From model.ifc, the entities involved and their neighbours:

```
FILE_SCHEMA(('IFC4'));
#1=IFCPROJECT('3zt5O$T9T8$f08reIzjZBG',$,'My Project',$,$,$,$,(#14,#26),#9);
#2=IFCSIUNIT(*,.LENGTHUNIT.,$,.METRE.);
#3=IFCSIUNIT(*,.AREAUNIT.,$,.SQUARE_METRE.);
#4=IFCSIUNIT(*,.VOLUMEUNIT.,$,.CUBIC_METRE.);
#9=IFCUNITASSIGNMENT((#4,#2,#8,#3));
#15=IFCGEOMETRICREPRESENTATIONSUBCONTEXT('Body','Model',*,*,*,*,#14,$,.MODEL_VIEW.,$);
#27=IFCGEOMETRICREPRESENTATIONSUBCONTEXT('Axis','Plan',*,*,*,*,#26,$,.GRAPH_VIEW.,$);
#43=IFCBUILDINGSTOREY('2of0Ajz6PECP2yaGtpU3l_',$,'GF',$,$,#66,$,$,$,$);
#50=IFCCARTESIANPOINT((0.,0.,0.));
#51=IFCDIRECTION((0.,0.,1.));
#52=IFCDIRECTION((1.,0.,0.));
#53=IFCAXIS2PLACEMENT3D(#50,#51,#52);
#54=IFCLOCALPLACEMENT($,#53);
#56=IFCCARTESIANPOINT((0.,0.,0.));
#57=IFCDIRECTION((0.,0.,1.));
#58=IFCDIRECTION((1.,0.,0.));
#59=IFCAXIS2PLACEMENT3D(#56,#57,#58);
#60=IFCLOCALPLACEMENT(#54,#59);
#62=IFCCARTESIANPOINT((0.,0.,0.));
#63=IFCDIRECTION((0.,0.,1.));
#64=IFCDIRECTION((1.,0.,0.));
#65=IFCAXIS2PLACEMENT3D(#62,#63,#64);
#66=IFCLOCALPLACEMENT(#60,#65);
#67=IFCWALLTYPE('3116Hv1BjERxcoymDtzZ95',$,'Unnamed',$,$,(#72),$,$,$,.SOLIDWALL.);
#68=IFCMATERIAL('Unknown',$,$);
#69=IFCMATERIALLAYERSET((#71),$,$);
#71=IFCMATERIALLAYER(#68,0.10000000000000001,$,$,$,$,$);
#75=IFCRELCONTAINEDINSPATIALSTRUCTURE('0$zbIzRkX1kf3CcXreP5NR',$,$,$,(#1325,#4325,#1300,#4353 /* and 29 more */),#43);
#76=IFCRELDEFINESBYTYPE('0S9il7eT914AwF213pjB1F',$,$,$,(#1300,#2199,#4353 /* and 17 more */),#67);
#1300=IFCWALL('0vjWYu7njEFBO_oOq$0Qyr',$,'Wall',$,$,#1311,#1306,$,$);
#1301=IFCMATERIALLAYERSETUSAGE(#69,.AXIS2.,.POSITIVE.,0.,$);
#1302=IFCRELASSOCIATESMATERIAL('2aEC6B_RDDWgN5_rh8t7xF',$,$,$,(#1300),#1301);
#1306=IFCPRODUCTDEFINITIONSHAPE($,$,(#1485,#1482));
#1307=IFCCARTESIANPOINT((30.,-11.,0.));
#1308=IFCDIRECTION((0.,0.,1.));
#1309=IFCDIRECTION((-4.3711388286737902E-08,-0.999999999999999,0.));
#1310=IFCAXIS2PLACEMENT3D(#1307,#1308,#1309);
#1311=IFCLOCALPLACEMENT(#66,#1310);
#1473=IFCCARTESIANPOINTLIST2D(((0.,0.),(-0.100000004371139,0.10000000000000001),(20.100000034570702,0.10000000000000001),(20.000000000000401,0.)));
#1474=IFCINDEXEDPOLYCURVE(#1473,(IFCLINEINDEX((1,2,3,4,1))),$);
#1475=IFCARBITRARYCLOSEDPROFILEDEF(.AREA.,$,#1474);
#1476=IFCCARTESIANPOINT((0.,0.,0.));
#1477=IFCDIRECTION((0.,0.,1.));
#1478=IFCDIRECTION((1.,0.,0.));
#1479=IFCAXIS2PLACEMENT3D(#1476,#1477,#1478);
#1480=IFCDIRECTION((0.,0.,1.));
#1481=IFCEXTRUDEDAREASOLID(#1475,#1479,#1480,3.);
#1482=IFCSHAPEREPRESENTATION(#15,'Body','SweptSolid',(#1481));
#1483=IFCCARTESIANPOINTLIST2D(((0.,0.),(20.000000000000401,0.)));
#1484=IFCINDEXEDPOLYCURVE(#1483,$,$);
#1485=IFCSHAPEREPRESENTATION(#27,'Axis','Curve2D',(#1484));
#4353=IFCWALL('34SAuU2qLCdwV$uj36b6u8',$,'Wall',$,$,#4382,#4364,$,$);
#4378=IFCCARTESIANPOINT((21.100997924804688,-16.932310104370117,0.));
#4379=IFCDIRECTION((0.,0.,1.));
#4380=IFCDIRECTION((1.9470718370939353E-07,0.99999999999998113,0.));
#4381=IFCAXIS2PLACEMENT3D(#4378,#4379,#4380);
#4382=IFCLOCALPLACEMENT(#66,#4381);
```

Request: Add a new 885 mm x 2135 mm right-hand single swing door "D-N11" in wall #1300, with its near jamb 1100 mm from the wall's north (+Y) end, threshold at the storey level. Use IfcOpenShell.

```python
import numpy as np
import ifcopenshell
import ifcopenshell.api.feature
import ifcopenshell.api.geometry
import ifcopenshell.api.root
import ifcopenshell.api.spatial
import ifcopenshell.geom
import ifcopenshell.util.element
import ifcopenshell.util.placement
import ifcopenshell.util.representation
import ifcopenshell.util.shape
import ifcopenshell.util.unit

model = ifcopenshell.open("model.ifc")
unit_scale = ifcopenshell.util.unit.calculate_unit_scale(model)
settings = ifcopenshell.geom.settings()


def volume(element):
    """Net volume in cubic metres, openings subtracted."""
    shape = ifcopenshell.geom.create_shape(settings, element)
    return ifcopenshell.util.shape.get_volume(shape.geometry)


wall = model.by_guid("0vjWYu7njEFBO_oOq$0Qyr")
storey = ifcopenshell.util.element.get_container(wall, ifc_class="IfcBuildingStorey")
context = ifcopenshell.util.representation.get_context(model, "Model", "Body", "MODEL_VIEW")
before = volume(wall)

width, height, from_end, sill = 0.885, 2.135, 1.1, 0.0  # metres

# The wall runs along its own X axis, and the end named is its -X end.
wall_shape = ifcopenshell.geom.create_shape(settings, wall)
x, y, z = ifcopenshell.util.shape.get_vertices(wall_shape.geometry).T
start = x.min() + from_end
face, thickness = float(y.min()), float(y.max() - y.min())
wall_matrix = ifcopenshell.util.placement.get_local_placement(wall.ObjectPlacement)
level = ifcopenshell.util.placement.get_local_placement(storey.ObjectPlacement)[2, 3]


def in_wall(x, y):
    """Placement at x, y metres in the wall's axes, at sill height."""
    matrix = wall_matrix.copy()
    matrix[:, 3] = wall_matrix @ np.array([x / unit_scale, y / unit_scale, 0.0, 1.0])
    matrix[2, 3] = level + sill / unit_scale
    return matrix


# Opening: a box that overshoots both wall faces by 50 mm.
opening = ifcopenshell.api.root.create_entity(model, ifc_class="IfcOpeningElement", predefined_type="OPENING")
box = ifcopenshell.api.geometry.add_wall_representation(
    model, context=context, length=width, height=height, thickness=thickness + 0.1
)
ifcopenshell.api.geometry.assign_representation(model, product=opening, representation=box)
ifcopenshell.api.geometry.edit_object_placement(model, product=opening, matrix=in_wall(start, face - 0.05), is_si=False)
ifcopenshell.api.feature.add_feature(model, feature=opening, element=wall)

door = ifcopenshell.api.root.create_entity(model, ifc_class="IfcDoor", name="D-N11", predefined_type="DOOR")
door.OverallWidth, door.OverallHeight = width / unit_scale, height / unit_scale
door.OperationType = "SINGLE_SWING_RIGHT"
body = ifcopenshell.api.geometry.add_door_representation(
    model,
    context=context,
    overall_width=door.OverallWidth,
    overall_height=door.OverallHeight,
    operation_type="SINGLE_SWING_RIGHT",
    lining_properties={"LiningDepth": thickness / unit_scale, "ThresholdDepth": thickness / unit_scale},
)
ifcopenshell.api.geometry.assign_representation(model, product=door, representation=body)
ifcopenshell.api.spatial.assign_container(model, products=[door], relating_structure=storey)
ifcopenshell.api.feature.add_filling(model, opening=opening, element=door)

# The lining spans the wall, so the door starts at the wall face.
ifcopenshell.api.geometry.edit_object_placement(model, product=door, matrix=in_wall(start, face), is_si=False)

after = volume(wall)

print(f"wall volume {before:.3f} -> {after:.3f} m3")

model.write("model_rev.ifc")
```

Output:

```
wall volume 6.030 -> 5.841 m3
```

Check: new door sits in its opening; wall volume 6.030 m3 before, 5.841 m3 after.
